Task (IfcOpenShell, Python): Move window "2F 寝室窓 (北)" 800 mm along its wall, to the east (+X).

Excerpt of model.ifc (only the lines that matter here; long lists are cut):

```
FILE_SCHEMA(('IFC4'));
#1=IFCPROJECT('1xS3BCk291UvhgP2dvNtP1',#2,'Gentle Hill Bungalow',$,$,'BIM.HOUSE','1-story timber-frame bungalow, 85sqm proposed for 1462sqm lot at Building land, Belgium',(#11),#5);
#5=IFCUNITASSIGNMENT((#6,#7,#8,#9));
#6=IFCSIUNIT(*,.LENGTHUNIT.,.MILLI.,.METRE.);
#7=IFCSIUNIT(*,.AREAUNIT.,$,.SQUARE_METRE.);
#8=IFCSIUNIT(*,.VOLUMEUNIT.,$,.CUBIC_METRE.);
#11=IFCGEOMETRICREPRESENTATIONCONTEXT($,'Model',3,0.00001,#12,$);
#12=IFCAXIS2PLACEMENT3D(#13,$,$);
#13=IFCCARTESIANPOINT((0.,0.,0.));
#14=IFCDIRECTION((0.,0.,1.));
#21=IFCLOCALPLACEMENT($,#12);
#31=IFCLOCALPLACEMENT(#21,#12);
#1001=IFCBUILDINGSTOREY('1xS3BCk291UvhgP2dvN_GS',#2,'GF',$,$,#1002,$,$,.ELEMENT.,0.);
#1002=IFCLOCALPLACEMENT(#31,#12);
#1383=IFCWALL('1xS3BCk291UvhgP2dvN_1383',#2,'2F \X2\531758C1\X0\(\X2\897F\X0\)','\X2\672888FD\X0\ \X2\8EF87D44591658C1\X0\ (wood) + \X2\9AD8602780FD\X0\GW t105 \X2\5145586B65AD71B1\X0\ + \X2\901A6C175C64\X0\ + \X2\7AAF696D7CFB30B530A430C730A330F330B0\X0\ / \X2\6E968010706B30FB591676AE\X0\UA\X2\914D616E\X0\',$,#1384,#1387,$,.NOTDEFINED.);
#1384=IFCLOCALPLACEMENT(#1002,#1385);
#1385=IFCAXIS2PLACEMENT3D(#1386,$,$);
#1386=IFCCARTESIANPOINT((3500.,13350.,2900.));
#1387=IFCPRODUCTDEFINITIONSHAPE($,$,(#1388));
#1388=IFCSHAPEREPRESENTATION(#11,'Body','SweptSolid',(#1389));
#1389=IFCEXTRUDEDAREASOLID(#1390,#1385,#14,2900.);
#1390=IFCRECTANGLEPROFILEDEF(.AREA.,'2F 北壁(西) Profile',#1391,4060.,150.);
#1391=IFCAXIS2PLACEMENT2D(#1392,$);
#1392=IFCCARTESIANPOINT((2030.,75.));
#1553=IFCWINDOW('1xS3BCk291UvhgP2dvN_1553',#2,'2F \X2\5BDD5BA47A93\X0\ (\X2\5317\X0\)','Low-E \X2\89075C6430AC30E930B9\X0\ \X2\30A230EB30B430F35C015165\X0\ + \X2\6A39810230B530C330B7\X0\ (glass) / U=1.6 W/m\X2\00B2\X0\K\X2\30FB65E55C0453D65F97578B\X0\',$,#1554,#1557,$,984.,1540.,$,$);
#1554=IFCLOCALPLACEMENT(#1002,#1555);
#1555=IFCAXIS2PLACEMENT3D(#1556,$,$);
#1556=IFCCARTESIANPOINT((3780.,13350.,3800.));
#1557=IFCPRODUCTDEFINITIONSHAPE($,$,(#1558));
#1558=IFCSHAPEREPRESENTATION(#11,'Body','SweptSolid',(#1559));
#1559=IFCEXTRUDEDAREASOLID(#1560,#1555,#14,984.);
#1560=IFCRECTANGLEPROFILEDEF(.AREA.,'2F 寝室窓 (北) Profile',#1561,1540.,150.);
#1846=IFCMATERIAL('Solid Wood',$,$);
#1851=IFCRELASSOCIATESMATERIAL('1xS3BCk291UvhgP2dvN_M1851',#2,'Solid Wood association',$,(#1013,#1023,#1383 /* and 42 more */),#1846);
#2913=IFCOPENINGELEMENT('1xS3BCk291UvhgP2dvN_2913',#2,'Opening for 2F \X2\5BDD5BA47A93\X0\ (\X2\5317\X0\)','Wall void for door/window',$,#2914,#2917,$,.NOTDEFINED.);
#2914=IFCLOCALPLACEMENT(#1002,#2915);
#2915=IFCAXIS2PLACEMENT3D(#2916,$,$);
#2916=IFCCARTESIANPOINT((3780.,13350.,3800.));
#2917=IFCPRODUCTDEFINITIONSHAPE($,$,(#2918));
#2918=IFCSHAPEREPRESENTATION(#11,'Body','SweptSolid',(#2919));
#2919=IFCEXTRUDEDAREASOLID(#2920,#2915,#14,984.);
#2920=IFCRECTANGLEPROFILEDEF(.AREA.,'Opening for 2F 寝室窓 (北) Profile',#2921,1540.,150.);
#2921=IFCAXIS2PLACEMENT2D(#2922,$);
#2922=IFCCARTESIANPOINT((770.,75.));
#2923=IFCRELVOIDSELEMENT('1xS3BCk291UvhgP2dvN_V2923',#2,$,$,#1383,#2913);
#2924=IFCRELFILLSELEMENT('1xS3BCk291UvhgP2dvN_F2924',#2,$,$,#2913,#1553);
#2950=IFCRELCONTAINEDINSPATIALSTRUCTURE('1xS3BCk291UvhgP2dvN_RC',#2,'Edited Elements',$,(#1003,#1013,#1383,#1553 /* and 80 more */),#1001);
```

```python
import ifcopenshell
import ifcopenshell.api.geometry
import ifcopenshell.util.placement

model = ifcopenshell.open("model.ifc")

window = model.by_guid("1xS3BCk291UvhgP2dvN_1553")
opening = window.FillsVoids[0].RelatingOpeningElement
wall = opening.VoidsElements[0].RelatingBuildingElement

wall_matrix = ifcopenshell.util.placement.get_local_placement(wall.ObjectPlacement)
shift = wall_matrix[:3, 0] * 800.0
before = ifcopenshell.util.placement.get_local_placement(window.ObjectPlacement)[:3, 3].copy()

# The window is not placed relative to its opening, so move both.
for product in (opening, window):
    matrix = ifcopenshell.util.placement.get_local_placement(product.ObjectPlacement)
    matrix[:3, 3] += shift
    ifcopenshell.api.geometry.edit_object_placement(model, product=product, matrix=matrix, is_si=False)

after = ifcopenshell.util.placement.get_local_placement(window.ObjectPlacement)[:3, 3]
print("window moved by", (after - before).round(3) + 0.0)

model.write("model_v2.ifc")
```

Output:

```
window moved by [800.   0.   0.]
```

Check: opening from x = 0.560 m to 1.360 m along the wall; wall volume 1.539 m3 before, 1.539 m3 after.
